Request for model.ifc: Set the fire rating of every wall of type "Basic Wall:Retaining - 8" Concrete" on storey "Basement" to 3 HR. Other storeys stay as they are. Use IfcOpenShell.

First a look at what the model holds.

```python
import ifcopenshell
import ifcopenshell.util.element

model = ifcopenshell.open("model.ifc")
print(model.schema)
storey = next(s for s in model.by_type("IfcBuildingStorey") if s.Name == "Basement")
walls = [e for e in ifcopenshell.util.element.get_decomposition(storey) if e.is_a("IfcWall")]
seen = {}
for e in walls:
    element_type = ifcopenshell.util.element.get_type(e)
    key = (element_type.Name if element_type != e and element_type else None, ifcopenshell.util.element.get_pset(e, "Pset_WallCommon", "FireRating"))
    seen[key] = seen.get(key, 0) + 1
for (name, value), count in sorted(seen.items(), key=str):
    print(count, "x", name, "|", value)
```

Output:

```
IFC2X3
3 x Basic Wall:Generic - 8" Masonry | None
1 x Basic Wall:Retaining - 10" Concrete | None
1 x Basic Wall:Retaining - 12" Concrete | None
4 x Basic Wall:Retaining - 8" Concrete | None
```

```python
import ifcopenshell
import ifcopenshell.api.pset
import ifcopenshell.util.element

model = ifcopenshell.open("model.ifc")

storey = next(s for s in model.by_type("IfcBuildingStorey") if s.Name == "Basement")
walls = [e for e in ifcopenshell.util.element.get_decomposition(storey) if e.is_a("IfcWall")]

count = 0
for e in walls:
    element_type = ifcopenshell.util.element.get_type(e)
    if element_type in (None, e) or element_type.Name != 'Basic Wall:Retaining - 8" Concrete':
        continue
    # add_pset returns the element's existing set when there is one.
    pset = ifcopenshell.api.pset.add_pset(model, product=e, name="Pset_WallCommon")
    ifcopenshell.api.pset.edit_pset(model, pset=pset, properties={"FireRating": "3 HR"})
    count += 1

print(count, "walls updated")

model.write("model-out.ifc")
```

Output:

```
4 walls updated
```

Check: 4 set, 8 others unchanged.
